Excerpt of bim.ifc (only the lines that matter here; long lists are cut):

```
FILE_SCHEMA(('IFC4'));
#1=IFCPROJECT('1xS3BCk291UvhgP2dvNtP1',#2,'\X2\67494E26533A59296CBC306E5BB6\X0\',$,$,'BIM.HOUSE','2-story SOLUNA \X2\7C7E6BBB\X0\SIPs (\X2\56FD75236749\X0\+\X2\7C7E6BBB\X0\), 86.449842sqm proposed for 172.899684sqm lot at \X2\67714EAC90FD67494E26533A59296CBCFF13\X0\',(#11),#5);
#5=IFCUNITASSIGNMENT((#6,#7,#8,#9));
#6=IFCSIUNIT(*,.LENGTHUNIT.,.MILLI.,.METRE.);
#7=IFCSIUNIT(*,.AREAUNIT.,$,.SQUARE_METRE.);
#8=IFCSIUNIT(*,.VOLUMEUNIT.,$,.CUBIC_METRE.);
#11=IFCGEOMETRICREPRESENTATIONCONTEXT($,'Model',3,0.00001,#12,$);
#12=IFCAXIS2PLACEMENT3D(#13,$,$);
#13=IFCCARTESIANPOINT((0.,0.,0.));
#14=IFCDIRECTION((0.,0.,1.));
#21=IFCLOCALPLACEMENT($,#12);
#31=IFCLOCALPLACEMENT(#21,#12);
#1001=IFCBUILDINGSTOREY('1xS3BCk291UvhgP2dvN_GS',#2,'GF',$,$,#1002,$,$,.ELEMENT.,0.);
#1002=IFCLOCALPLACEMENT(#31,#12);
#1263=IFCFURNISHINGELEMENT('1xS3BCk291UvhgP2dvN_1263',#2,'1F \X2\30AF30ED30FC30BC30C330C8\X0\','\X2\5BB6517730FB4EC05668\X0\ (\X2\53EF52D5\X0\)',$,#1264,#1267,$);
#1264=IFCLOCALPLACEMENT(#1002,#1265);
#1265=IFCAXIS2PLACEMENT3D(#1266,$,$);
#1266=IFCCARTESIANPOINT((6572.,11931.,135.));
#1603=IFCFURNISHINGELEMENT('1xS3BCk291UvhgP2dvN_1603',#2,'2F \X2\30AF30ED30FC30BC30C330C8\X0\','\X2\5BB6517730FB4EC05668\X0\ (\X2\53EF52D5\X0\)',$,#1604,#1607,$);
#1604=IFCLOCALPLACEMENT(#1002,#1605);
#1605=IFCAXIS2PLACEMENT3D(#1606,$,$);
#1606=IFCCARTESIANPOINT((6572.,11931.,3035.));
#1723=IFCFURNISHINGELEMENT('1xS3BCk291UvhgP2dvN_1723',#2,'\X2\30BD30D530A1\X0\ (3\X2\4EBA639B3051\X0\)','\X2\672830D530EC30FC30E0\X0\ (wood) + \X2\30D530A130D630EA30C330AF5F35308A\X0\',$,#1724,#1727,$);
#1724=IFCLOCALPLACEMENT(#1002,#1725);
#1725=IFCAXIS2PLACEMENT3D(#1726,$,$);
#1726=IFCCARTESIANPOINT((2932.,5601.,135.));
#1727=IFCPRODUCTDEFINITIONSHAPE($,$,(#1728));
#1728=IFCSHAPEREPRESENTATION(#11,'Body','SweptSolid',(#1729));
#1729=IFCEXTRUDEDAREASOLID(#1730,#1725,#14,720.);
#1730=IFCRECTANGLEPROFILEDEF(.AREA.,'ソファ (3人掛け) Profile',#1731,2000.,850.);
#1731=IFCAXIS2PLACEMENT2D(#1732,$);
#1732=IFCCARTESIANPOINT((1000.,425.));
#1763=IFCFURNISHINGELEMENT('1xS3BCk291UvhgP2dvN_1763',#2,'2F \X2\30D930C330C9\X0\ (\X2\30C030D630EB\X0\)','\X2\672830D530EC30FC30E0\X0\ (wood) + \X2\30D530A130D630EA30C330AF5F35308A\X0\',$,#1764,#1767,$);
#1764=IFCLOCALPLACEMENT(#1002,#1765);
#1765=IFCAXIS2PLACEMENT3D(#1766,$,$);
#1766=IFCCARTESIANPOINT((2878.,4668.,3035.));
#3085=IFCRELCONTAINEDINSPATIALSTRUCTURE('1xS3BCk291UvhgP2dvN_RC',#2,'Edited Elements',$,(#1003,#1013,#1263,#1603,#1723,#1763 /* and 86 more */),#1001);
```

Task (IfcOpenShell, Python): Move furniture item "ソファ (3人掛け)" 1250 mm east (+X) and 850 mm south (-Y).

```python
import ifcopenshell
import ifcopenshell.api.geometry
import ifcopenshell.util.placement

model = ifcopenshell.open("bim.ifc")

item = model.by_guid("1xS3BCk291UvhgP2dvN_1723")
matrix = ifcopenshell.util.placement.get_local_placement(item.ObjectPlacement)
matrix[0, 3] += 1250.0
matrix[1, 3] -= 850.0
ifcopenshell.api.geometry.edit_object_placement(model, product=item, matrix=matrix, is_si=False)

print(ifcopenshell.util.placement.get_local_placement(item.ObjectPlacement).round(3) + 0.0)

model.write("bim_rev.ifc")
```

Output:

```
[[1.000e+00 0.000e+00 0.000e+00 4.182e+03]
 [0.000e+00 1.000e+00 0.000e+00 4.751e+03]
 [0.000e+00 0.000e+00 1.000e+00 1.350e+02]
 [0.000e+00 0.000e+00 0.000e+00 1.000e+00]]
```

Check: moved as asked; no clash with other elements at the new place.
